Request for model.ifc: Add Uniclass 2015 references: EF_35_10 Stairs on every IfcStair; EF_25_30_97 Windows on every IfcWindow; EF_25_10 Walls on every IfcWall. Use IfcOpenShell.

First a look at what the model holds.

```python
import ifcopenshell

model = ifcopenshell.open("model.ifc")
print(model.schema)
print("classifications:", [c.Name for c in model.by_type("IfcClassification")])
for ifc_class in ("IfcDoor", "IfcRoof", "IfcStair", "IfcWall", "IfcWindow"):
    print(ifc_class, len(model.by_type(ifc_class)))
```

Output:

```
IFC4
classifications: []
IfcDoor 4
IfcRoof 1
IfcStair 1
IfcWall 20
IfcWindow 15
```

```python
import ifcopenshell
import ifcopenshell.api.classification

model = ifcopenshell.open("model.ifc")

system = ifcopenshell.api.classification.add_classification(model, classification="Uniclass 2015")

codes = {
    "IfcStair": ("EF_35_10", "Stairs"),
    "IfcWindow": ("EF_25_30_97", "Windows"),
    "IfcWall": ("EF_25_10", "Walls"),
}
for ifc_class, (code, name) in codes.items():
    products = model.by_type(ifc_class)
    ifcopenshell.api.classification.add_reference(
        model, products=products, classification=system, identification=code, name=name
    )
    print(code, len(products))

model.write("model_edited.ifc")
```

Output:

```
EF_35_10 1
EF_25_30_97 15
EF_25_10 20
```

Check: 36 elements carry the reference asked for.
